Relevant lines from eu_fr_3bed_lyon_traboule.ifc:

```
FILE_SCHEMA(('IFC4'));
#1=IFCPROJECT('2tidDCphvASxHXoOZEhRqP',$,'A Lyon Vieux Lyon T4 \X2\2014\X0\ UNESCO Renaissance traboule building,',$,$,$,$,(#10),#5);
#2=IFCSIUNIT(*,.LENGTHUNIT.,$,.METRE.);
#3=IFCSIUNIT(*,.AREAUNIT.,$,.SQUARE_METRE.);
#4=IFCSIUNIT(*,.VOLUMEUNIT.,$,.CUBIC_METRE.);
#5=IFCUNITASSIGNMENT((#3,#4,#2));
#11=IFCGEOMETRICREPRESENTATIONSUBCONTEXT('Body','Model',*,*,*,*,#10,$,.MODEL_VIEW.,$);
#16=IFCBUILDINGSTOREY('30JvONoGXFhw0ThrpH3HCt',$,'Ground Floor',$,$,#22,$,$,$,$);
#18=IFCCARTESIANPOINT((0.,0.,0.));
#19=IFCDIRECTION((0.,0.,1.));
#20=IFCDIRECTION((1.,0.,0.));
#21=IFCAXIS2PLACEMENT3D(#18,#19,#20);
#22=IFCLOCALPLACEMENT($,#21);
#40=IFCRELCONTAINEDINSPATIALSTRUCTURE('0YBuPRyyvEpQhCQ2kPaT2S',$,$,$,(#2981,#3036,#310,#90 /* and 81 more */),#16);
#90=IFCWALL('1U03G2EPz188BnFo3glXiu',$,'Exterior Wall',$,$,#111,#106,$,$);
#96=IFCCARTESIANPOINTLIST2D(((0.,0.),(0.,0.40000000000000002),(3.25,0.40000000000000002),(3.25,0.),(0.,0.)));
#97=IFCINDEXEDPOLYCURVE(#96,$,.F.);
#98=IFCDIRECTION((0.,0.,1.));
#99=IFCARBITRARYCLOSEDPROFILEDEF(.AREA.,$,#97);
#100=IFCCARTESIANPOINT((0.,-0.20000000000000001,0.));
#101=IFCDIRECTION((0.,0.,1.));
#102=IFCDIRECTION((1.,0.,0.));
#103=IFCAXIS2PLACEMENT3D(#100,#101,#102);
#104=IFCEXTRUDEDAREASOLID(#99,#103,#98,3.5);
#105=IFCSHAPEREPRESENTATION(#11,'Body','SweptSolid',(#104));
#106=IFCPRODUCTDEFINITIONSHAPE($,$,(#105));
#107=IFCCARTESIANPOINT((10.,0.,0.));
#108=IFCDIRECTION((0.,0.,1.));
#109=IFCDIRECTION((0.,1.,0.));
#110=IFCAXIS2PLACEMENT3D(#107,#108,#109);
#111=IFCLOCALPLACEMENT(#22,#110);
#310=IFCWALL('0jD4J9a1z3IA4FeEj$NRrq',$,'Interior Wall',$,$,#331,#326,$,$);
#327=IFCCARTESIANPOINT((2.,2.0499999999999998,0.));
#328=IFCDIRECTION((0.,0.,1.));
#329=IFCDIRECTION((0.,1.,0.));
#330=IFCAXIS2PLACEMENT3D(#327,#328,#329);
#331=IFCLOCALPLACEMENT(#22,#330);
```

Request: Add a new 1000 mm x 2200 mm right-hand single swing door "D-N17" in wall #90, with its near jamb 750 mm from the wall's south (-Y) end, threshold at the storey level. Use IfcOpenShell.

```python
import numpy as np
import ifcopenshell
import ifcopenshell.api.feature
import ifcopenshell.api.geometry
import ifcopenshell.api.root
import ifcopenshell.api.spatial
import ifcopenshell.geom
import ifcopenshell.util.element
import ifcopenshell.util.placement
import ifcopenshell.util.representation
import ifcopenshell.util.shape
import ifcopenshell.util.unit

model = ifcopenshell.open("eu_fr_3bed_lyon_traboule.ifc")
unit_scale = ifcopenshell.util.unit.calculate_unit_scale(model)
settings = ifcopenshell.geom.settings()


def volume(element):
    """Net volume in cubic metres, openings subtracted."""
    shape = ifcopenshell.geom.create_shape(settings, element)
    return ifcopenshell.util.shape.get_volume(shape.geometry)


wall = model.by_guid("1U03G2EPz188BnFo3glXiu")
storey = ifcopenshell.util.element.get_container(wall, ifc_class="IfcBuildingStorey")
context = ifcopenshell.util.representation.get_context(model, "Model", "Body", "MODEL_VIEW")
before = volume(wall)

width, height, from_end, sill = 1, 2.2, 0.75, 0.0  # metres

# The wall runs along its own X axis, and the end named is its -X end.
wall_shape = ifcopenshell.geom.create_shape(settings, wall)
x, y, z = ifcopenshell.util.shape.get_vertices(wall_shape.geometry).T
start = x.min() + from_end
face, thickness = float(y.min()), float(y.max() - y.min())
wall_matrix = ifcopenshell.util.placement.get_local_placement(wall.ObjectPlacement)
level = ifcopenshell.util.placement.get_local_placement(storey.ObjectPlacement)[2, 3]


def in_wall(x, y):
    """Placement at x, y metres in the wall's axes, at sill height."""
    matrix = wall_matrix.copy()
    matrix[:, 3] = wall_matrix @ np.array([x / unit_scale, y / unit_scale, 0.0, 1.0])
    matrix[2, 3] = level + sill / unit_scale
    return matrix


# Opening: a box that overshoots both wall faces by 50 mm.
opening = ifcopenshell.api.root.create_entity(model, ifc_class="IfcOpeningElement", predefined_type="OPENING")
box = ifcopenshell.api.geometry.add_wall_representation(
    model, context=context, length=width, height=height, thickness=thickness + 0.1
)
ifcopenshell.api.geometry.assign_representation(model, product=opening, representation=box)
ifcopenshell.api.geometry.edit_object_placement(model, product=opening, matrix=in_wall(start, face - 0.05), is_si=False)
ifcopenshell.api.feature.add_feature(model, feature=opening, element=wall)

door = ifcopenshell.api.root.create_entity(model, ifc_class="IfcDoor", name="D-N17", predefined_type="DOOR")
door.OverallWidth, door.OverallHeight = width / unit_scale, height / unit_scale
door.OperationType = "SINGLE_SWING_RIGHT"
body = ifcopenshell.api.geometry.add_door_representation(
    model,
    context=context,
    overall_width=door.OverallWidth,
    overall_height=door.OverallHeight,
    operation_type="SINGLE_SWING_RIGHT",
    lining_properties={"LiningDepth": thickness / unit_scale, "ThresholdDepth": thickness / unit_scale},
)
ifcopenshell.api.geometry.assign_representation(model, product=door, representation=body)
ifcopenshell.api.spatial.assign_container(model, products=[door], relating_structure=storey)
ifcopenshell.api.feature.add_filling(model, opening=opening, element=door)

# The lining spans the wall, so the door starts at the wall face.
ifcopenshell.api.geometry.edit_object_placement(model, product=door, matrix=in_wall(start, face), is_si=False)

after = volume(wall)

print(f"wall volume {before:.3f} -> {after:.3f} m3")

model.write("eu_fr_3bed_lyon_traboule-out.ifc")
```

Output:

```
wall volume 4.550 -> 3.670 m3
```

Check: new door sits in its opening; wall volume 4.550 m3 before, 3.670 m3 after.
